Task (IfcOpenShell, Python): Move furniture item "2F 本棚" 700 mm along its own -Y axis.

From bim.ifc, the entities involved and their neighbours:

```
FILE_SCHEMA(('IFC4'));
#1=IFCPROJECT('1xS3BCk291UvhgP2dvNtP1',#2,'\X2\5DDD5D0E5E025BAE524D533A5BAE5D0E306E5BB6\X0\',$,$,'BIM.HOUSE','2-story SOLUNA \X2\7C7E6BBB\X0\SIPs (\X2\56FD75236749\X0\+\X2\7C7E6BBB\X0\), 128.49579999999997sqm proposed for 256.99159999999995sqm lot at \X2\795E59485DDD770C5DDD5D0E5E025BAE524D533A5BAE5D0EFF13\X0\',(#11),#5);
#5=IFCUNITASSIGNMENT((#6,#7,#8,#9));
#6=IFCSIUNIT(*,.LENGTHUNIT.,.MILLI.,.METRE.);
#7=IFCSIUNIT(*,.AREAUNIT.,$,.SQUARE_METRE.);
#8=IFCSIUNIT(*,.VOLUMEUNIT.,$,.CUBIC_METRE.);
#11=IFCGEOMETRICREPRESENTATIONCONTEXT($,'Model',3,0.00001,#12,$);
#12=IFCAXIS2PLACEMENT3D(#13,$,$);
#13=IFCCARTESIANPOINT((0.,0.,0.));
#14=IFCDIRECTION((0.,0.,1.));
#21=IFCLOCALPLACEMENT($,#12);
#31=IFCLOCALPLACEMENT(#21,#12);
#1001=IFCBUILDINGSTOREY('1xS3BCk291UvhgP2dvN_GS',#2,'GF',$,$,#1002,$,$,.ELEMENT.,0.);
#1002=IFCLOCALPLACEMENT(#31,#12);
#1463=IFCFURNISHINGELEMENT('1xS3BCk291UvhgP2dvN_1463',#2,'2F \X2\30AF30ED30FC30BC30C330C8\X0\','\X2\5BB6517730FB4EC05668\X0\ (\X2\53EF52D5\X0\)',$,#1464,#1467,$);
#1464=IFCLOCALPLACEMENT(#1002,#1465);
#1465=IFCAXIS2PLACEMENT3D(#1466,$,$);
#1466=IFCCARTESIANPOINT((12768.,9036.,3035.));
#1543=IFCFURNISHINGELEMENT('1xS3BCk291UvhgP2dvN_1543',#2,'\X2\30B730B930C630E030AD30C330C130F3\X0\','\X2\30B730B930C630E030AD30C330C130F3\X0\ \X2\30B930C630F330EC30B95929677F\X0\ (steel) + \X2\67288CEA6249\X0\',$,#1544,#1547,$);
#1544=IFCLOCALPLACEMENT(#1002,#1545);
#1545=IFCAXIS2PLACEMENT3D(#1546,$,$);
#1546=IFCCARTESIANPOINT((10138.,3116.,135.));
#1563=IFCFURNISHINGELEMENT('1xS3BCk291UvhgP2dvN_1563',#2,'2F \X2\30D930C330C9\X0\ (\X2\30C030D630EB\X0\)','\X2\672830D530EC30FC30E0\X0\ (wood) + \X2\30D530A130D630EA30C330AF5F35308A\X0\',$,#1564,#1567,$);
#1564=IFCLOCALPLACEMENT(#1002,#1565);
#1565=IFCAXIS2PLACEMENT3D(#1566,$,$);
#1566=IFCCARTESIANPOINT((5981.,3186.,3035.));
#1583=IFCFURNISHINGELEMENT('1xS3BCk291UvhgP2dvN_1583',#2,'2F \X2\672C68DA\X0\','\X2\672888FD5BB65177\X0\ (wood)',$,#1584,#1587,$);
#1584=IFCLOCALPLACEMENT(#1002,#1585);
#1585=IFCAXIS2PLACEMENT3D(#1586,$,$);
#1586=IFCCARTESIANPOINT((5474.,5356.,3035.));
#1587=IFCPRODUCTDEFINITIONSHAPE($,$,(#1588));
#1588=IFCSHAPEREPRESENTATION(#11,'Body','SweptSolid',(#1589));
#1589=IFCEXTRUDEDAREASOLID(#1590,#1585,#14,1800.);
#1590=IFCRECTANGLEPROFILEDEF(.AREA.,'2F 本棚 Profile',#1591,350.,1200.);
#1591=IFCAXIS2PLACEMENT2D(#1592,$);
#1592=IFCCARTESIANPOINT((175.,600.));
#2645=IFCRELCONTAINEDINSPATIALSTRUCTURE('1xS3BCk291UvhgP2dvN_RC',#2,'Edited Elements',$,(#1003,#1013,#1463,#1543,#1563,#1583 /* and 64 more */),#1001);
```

```python
import ifcopenshell
import ifcopenshell.api.geometry
import ifcopenshell.util.placement
import ifcopenshell.util.unit

model = ifcopenshell.open("bim.ifc")
unit_scale = ifcopenshell.util.unit.calculate_unit_scale(model)

item = model.by_guid("1xS3BCk291UvhgP2dvN_1583")
matrix = ifcopenshell.util.placement.get_local_placement(item.ObjectPlacement)
matrix[:3, 3] -= matrix[:3, 1] * 0.7 / unit_scale
ifcopenshell.api.geometry.edit_object_placement(model, product=item, matrix=matrix, is_si=False)

print(ifcopenshell.util.placement.get_local_placement(item.ObjectPlacement).round(3) + 0.0)

model.write("bim_rev.ifc")
```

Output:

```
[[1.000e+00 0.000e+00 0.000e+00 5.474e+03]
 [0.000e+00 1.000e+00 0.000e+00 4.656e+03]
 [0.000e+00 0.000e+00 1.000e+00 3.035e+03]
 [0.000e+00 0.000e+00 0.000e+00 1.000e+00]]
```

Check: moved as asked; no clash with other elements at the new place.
